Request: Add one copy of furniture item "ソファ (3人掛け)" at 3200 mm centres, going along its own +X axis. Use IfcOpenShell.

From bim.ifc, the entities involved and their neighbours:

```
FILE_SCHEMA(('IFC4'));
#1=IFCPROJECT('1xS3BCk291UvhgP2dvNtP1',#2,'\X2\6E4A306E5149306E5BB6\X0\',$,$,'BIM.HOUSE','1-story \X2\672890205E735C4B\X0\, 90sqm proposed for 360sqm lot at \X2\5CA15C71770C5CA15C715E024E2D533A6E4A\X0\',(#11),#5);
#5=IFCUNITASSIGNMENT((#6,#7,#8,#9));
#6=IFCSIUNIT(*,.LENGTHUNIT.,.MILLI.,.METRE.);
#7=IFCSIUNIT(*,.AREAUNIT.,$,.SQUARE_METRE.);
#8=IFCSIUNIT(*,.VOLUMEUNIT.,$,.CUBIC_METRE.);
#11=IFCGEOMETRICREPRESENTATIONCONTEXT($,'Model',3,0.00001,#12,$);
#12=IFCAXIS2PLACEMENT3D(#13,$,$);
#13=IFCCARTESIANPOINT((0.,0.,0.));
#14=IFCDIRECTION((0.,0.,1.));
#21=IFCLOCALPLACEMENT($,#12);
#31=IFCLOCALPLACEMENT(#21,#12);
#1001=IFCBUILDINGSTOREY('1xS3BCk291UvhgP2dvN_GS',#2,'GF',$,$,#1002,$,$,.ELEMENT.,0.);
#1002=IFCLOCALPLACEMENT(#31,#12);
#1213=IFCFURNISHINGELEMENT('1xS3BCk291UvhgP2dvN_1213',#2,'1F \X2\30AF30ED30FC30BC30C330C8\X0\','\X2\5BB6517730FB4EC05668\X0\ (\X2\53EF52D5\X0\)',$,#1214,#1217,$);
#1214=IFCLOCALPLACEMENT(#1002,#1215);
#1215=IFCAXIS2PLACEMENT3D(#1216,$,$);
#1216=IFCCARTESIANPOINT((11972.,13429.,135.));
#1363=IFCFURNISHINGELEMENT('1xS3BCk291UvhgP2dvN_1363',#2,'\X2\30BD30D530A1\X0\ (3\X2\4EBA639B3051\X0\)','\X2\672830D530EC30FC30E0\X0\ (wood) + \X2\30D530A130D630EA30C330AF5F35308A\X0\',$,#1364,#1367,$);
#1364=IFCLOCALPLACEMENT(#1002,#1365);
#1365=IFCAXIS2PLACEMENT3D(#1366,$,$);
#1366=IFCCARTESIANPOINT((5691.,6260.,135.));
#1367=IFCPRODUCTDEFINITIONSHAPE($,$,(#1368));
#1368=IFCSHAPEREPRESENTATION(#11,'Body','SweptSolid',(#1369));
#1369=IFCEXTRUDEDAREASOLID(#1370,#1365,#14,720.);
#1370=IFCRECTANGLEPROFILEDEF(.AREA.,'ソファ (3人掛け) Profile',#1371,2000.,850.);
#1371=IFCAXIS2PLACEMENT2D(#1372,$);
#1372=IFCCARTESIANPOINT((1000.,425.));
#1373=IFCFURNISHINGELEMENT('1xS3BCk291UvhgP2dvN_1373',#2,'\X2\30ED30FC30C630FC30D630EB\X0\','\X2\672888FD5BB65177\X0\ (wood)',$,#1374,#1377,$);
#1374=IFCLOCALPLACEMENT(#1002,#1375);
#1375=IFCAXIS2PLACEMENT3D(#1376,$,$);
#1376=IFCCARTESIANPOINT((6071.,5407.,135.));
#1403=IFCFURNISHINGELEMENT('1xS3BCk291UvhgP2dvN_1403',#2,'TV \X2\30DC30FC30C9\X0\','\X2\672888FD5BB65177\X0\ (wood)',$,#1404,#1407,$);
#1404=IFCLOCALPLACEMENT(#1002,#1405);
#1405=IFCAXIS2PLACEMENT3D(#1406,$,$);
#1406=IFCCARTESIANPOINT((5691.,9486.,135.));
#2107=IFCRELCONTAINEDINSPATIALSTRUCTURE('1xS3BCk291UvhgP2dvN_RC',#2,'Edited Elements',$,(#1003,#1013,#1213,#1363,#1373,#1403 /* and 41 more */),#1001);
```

```python
import ifcopenshell
import ifcopenshell.api.geometry
import ifcopenshell.api.root
import ifcopenshell.util.element
import ifcopenshell.util.placement
import ifcopenshell.util.unit

model = ifcopenshell.open("bim.ifc")
unit_scale = ifcopenshell.util.unit.calculate_unit_scale(model)


def reuse_history(source, copy):
    """copy_class also copies each property set's owner history, people and application; keep the originals."""
    for rel in copy.IsDefinedBy:
        if rel.is_a("IfcRelDefinesByProperties") and (history := rel.RelatingPropertyDefinition.OwnerHistory):
            rel.RelatingPropertyDefinition.OwnerHistory = source.OwnerHistory
            ifcopenshell.util.element.remove_deep2(model, history)


source = model.by_guid("1xS3BCk291UvhgP2dvN_1363")
base = ifcopenshell.util.placement.get_local_placement(source.ObjectPlacement)
step = base[:3, 0] * 3.2 / unit_scale

for i in range(1, 2):
    copy = ifcopenshell.api.root.copy_class(model, product=source)
    copy.Representation = ifcopenshell.util.element.copy_deep(
        model, source.Representation, exclude=["IfcGeometricRepresentationContext", "IfcRepresentationMap"]
    )
    reuse_history(source, copy)
    matrix = base.copy()
    matrix[:3, 3] += i * step
    print("added at", matrix[:3, 3].round(3) + 0.0)
    ifcopenshell.api.geometry.edit_object_placement(model, product=copy, matrix=matrix, is_si=False)

model.write("bim_rev.ifc")
```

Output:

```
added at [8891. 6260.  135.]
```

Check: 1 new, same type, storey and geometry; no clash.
